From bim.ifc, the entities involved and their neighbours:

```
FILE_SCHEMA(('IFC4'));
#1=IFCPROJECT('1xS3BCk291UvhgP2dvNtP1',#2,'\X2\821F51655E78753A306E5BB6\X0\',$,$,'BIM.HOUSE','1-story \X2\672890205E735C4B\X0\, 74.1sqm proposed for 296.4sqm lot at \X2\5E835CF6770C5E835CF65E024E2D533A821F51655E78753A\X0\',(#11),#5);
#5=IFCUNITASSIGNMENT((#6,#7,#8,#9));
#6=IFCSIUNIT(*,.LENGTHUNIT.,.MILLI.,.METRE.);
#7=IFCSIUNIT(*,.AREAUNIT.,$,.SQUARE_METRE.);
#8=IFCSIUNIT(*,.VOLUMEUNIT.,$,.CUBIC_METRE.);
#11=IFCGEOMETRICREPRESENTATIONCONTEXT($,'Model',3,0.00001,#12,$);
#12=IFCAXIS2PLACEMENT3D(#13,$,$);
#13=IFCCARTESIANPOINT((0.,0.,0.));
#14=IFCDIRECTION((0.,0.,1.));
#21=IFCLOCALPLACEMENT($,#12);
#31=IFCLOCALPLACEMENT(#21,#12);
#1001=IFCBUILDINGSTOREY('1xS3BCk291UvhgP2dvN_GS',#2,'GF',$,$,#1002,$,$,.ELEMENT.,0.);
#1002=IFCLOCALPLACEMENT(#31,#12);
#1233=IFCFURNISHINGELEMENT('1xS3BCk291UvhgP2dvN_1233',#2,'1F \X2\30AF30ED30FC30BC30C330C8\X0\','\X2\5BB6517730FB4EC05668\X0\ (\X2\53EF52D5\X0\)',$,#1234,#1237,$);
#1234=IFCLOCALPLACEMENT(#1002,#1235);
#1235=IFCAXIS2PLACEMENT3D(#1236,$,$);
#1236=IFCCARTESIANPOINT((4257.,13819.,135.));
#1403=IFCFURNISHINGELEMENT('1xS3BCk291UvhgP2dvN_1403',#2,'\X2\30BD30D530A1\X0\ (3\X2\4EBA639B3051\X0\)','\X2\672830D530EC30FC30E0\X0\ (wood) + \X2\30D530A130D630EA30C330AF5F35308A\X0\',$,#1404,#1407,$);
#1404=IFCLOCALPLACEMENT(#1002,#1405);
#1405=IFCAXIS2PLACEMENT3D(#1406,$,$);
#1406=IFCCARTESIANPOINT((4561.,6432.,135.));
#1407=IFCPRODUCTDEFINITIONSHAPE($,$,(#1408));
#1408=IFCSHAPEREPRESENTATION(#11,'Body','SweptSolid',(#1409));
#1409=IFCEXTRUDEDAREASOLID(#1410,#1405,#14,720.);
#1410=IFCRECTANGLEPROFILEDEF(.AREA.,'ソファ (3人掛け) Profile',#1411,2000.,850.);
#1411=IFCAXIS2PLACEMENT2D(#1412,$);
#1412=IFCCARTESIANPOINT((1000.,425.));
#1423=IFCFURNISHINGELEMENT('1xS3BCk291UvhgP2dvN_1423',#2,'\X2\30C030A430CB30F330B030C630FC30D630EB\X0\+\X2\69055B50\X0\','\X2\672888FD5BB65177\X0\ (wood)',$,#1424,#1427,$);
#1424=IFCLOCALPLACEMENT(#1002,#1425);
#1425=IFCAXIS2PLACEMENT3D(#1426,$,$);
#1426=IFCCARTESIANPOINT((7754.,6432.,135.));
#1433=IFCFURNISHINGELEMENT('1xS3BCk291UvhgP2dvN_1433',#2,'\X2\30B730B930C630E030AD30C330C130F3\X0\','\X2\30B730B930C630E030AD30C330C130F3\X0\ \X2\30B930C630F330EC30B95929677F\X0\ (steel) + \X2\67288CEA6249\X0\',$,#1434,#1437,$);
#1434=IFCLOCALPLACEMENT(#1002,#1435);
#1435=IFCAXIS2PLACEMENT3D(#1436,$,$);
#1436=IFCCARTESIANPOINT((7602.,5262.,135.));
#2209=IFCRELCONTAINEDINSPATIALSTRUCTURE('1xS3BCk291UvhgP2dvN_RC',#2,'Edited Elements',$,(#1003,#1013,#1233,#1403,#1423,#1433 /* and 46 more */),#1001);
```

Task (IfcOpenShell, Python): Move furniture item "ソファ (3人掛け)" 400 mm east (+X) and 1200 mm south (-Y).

```python
import ifcopenshell
import ifcopenshell.api.geometry
import ifcopenshell.util.placement
import ifcopenshell.util.unit

model = ifcopenshell.open("bim.ifc")
unit_scale = ifcopenshell.util.unit.calculate_unit_scale(model)

item = model.by_id(1403)
matrix = ifcopenshell.util.placement.get_local_placement(item.ObjectPlacement)
matrix[0, 3] += 0.4 / unit_scale
matrix[1, 3] -= 1.2 / unit_scale
ifcopenshell.api.geometry.edit_object_placement(model, product=item, matrix=matrix, is_si=False)

print(ifcopenshell.util.placement.get_local_placement(item.ObjectPlacement).round(3) + 0.0)

model.write("bim_updated.ifc")
```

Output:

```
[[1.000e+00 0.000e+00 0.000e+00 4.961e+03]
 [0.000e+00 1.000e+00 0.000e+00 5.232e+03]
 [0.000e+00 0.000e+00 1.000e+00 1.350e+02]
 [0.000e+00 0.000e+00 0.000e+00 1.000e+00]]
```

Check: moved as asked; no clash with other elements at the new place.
